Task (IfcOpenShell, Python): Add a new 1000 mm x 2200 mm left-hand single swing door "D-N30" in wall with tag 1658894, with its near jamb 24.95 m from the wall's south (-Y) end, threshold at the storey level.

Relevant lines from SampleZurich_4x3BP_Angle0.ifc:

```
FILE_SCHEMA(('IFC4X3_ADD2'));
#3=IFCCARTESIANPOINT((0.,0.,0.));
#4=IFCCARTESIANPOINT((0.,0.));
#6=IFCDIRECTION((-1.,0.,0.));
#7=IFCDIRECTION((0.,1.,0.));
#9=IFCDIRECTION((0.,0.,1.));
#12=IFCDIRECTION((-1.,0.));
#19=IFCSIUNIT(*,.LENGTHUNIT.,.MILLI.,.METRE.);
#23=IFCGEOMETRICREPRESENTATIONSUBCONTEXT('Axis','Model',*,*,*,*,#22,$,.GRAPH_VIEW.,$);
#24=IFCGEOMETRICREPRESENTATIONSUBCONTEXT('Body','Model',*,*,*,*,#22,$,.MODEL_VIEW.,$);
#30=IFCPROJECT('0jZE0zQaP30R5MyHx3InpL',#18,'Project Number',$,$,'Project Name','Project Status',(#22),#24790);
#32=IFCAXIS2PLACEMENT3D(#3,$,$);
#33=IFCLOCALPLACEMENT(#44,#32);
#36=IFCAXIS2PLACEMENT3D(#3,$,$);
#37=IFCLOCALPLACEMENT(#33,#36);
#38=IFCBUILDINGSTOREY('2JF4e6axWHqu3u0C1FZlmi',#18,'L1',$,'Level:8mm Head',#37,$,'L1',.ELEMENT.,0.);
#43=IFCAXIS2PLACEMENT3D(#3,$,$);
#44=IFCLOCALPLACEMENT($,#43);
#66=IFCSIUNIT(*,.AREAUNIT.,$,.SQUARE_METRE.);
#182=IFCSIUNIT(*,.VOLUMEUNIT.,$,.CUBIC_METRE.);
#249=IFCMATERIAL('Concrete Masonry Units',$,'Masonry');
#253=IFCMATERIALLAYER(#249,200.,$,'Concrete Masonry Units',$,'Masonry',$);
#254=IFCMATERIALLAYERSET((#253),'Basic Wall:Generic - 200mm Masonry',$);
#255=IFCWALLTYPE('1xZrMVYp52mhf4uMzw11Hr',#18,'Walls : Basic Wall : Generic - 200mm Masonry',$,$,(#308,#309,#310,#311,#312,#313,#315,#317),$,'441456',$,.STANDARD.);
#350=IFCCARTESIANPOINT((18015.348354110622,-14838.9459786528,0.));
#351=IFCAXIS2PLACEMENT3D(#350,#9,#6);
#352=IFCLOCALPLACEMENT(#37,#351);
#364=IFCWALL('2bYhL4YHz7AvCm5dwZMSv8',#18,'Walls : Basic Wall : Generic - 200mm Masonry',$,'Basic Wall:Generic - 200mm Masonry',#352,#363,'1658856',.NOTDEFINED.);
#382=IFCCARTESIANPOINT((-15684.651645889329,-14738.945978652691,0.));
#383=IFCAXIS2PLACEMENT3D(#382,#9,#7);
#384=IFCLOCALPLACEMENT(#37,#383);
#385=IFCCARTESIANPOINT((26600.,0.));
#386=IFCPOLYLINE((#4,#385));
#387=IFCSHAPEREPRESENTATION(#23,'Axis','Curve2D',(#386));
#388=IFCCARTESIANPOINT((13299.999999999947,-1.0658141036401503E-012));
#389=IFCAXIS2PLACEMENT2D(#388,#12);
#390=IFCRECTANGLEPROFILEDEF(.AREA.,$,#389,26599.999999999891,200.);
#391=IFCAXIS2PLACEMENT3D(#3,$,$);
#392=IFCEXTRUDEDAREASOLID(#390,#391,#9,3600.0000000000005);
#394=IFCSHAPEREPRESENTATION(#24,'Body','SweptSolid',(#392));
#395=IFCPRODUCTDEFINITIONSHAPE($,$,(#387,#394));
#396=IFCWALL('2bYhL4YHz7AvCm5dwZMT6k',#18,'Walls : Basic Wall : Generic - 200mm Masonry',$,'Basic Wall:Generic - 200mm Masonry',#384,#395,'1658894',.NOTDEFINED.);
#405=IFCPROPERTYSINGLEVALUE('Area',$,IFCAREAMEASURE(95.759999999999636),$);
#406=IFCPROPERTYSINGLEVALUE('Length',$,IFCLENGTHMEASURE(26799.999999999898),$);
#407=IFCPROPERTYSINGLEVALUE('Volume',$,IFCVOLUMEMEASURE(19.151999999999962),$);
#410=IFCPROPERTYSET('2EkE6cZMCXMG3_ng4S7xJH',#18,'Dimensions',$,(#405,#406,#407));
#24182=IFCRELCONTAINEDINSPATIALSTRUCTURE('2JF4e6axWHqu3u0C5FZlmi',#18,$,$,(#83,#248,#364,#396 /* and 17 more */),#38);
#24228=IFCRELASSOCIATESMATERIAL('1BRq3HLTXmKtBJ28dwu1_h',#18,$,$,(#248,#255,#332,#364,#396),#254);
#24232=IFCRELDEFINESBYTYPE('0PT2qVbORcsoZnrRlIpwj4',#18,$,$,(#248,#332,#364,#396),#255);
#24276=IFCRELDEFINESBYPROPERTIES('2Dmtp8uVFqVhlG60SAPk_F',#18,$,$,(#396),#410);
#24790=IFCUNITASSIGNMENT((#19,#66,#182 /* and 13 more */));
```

```python
import numpy as np
import ifcopenshell
import ifcopenshell.api.feature
import ifcopenshell.api.geometry
import ifcopenshell.api.pset
import ifcopenshell.api.root
import ifcopenshell.api.spatial
import ifcopenshell.geom
import ifcopenshell.util.element
import ifcopenshell.util.placement
import ifcopenshell.util.representation
import ifcopenshell.util.shape
import ifcopenshell.util.unit

model = ifcopenshell.open("SampleZurich_4x3BP_Angle0.ifc")
unit_scale = ifcopenshell.util.unit.calculate_unit_scale(model)
area_scale = ifcopenshell.util.unit.calculate_unit_scale(model, "AREAUNIT")
volume_scale = ifcopenshell.util.unit.calculate_unit_scale(model, "VOLUMEUNIT")
settings = ifcopenshell.geom.settings()


def volume(element):
    """Net volume in cubic metres, openings subtracted."""
    shape = ifcopenshell.geom.create_shape(settings, element)
    return ifcopenshell.util.shape.get_volume(shape.geometry)


wall = model.by_guid("2bYhL4YHz7AvCm5dwZMT6k")
storey = ifcopenshell.util.element.get_container(wall, ifc_class="IfcBuildingStorey")
context = ifcopenshell.util.representation.get_context(model, "Model", "Body", "MODEL_VIEW")
before = volume(wall)

width, height, from_end, sill = 1, 2.2, 24.95, 0.0  # metres

# The wall runs along its own X axis, and the end named is its -X end.
wall_shape = ifcopenshell.geom.create_shape(settings, wall)
x, y, z = ifcopenshell.util.shape.get_vertices(wall_shape.geometry).T
start = x.min() + from_end
face, thickness = float(y.min()), float(y.max() - y.min())
wall_matrix = ifcopenshell.util.placement.get_local_placement(wall.ObjectPlacement)
level = ifcopenshell.util.placement.get_local_placement(storey.ObjectPlacement)[2, 3]


def in_wall(x, y):
    """Placement at x, y metres in the wall's axes, at sill height."""
    matrix = wall_matrix.copy()
    matrix[:, 3] = wall_matrix @ np.array([x / unit_scale, y / unit_scale, 0.0, 1.0])
    matrix[2, 3] = level + sill / unit_scale
    return matrix


# Opening: a box that overshoots both wall faces by 50 mm.
opening = ifcopenshell.api.root.create_entity(model, ifc_class="IfcOpeningElement", predefined_type="OPENING")
box = ifcopenshell.api.geometry.add_wall_representation(
    model, context=context, length=width, height=height, thickness=thickness + 0.1
)
ifcopenshell.api.geometry.assign_representation(model, product=opening, representation=box)
ifcopenshell.api.geometry.edit_object_placement(model, product=opening, matrix=in_wall(start, face - 0.05), is_si=False)
ifcopenshell.api.feature.add_feature(model, feature=opening, element=wall)

door = ifcopenshell.api.root.create_entity(model, ifc_class="IfcDoor", name="D-N30", predefined_type="DOOR")
door.OverallWidth, door.OverallHeight = width / unit_scale, height / unit_scale
door.OperationType = "SINGLE_SWING_LEFT"
body = ifcopenshell.api.geometry.add_door_representation(
    model,
    context=context,
    overall_width=door.OverallWidth,
    overall_height=door.OverallHeight,
    operation_type="SINGLE_SWING_LEFT",
    lining_properties={"LiningDepth": thickness / unit_scale, "ThresholdDepth": thickness / unit_scale},
)
ifcopenshell.api.geometry.assign_representation(model, product=door, representation=body)
ifcopenshell.api.spatial.assign_container(model, products=[door], relating_structure=storey)
ifcopenshell.api.feature.add_filling(model, opening=opening, element=door)

# The lining spans the wall, so the door starts at the wall face.
ifcopenshell.api.geometry.edit_object_placement(model, product=door, matrix=in_wall(start, face), is_si=False)

after = volume(wall)

# Update the wall's stored quantities.
pset = model.by_id(ifcopenshell.util.element.get_pset(wall, "Dimensions", should_inherit=False)["id"])
ifcopenshell.api.pset.edit_pset(model, pset=pset, properties={
    "Area": model.create_entity("IfcAreaMeasure", after / thickness / area_scale),
    "Volume": model.create_entity("IfcVolumeMeasure", after / volume_scale),
})

print(f"wall volume {before:.3f} -> {after:.3f} m3")

model.write("SampleZurich_4x3BP_Angle0_v2.ifc")
```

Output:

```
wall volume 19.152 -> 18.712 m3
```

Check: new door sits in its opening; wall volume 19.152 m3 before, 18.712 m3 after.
